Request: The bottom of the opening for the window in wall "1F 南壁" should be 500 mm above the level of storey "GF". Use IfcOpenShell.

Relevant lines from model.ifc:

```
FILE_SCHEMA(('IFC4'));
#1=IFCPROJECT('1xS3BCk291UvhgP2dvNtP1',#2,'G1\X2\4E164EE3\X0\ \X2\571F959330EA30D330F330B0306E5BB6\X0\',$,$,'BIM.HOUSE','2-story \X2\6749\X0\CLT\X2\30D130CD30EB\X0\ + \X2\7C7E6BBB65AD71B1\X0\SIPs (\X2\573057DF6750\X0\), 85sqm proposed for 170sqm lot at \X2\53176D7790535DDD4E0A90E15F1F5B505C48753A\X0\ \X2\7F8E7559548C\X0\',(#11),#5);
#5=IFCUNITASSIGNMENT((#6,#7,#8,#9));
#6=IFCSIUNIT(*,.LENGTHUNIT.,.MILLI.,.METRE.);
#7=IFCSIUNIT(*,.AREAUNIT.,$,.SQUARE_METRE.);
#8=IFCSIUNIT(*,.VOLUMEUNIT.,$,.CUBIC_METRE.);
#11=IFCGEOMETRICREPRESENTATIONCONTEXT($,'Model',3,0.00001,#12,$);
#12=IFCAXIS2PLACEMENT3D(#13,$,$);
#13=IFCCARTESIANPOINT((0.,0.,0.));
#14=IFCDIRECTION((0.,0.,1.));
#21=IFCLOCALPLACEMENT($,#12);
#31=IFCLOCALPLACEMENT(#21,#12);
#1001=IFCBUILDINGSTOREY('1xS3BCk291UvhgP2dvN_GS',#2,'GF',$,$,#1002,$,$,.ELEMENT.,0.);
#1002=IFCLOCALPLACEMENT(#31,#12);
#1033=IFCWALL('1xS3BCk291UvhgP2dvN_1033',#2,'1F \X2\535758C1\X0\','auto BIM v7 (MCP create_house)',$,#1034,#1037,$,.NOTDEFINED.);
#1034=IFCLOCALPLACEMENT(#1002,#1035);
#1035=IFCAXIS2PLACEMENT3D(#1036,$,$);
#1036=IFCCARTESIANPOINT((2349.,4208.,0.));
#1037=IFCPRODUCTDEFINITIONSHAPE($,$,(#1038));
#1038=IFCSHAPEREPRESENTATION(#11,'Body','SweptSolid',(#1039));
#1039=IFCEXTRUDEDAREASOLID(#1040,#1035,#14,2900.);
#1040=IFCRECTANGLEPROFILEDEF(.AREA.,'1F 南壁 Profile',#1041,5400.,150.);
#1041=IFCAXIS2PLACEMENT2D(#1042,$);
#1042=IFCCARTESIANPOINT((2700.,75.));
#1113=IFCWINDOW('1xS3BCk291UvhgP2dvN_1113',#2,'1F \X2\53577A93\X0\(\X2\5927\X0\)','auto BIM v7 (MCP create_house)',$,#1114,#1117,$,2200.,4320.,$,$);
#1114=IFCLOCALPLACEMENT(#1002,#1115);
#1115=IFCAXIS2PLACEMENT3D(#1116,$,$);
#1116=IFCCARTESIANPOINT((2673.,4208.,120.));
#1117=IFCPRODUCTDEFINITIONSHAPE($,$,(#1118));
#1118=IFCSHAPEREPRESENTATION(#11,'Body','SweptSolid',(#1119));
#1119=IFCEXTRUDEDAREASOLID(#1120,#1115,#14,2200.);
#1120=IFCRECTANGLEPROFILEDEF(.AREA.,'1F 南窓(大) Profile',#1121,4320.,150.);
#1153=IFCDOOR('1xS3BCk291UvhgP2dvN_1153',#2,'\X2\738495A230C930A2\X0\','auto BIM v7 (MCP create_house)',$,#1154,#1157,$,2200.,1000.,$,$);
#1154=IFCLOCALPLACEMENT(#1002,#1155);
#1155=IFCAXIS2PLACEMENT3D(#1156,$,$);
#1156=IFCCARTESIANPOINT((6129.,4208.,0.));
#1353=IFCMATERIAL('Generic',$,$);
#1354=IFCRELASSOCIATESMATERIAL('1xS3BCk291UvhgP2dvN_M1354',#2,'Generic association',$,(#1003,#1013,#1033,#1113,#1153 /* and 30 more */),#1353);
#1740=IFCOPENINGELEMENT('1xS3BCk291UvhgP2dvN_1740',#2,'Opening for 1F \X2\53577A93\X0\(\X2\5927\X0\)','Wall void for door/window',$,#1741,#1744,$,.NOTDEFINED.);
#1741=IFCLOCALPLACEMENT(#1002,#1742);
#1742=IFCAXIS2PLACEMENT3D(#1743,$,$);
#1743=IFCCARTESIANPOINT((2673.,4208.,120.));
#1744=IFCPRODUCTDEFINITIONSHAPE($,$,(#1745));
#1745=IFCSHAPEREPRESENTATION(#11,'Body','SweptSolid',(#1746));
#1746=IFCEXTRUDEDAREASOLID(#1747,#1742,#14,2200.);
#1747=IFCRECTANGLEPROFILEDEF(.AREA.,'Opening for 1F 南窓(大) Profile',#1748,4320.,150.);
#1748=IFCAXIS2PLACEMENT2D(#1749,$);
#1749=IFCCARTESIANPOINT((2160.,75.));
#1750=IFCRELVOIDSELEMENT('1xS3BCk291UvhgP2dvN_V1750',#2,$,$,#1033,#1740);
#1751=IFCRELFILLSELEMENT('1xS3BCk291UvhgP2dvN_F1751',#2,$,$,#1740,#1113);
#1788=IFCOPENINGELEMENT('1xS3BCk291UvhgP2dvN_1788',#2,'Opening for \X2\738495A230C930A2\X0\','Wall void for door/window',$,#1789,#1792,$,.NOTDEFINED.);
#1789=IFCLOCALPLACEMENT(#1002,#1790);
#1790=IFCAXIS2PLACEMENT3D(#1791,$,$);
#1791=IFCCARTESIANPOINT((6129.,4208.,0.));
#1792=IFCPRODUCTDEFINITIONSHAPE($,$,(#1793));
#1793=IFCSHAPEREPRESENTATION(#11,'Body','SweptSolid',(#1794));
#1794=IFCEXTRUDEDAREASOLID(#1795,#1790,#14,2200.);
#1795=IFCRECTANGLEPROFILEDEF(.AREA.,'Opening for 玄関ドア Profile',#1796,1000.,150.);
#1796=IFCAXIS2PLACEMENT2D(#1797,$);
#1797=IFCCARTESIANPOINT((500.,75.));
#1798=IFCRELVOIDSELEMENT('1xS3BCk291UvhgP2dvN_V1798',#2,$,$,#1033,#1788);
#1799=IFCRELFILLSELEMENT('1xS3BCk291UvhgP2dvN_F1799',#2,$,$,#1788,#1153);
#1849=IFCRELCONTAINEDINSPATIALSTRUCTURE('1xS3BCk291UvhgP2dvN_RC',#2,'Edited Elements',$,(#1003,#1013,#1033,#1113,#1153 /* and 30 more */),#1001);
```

```python
import numpy as np
import ifcopenshell
import ifcopenshell.api.geometry
import ifcopenshell.geom
import ifcopenshell.util.element
import ifcopenshell.util.placement
import ifcopenshell.util.shape
import ifcopenshell.util.unit

model = ifcopenshell.open("model.ifc")
unit_scale = ifcopenshell.util.unit.calculate_unit_scale(model)

window = model.by_id(1113)
opening = window.FillsVoids[0].RelatingOpeningElement
storey = ifcopenshell.util.element.get_container(window, ifc_class="IfcBuildingStorey")
level = ifcopenshell.util.placement.get_local_placement(storey.ObjectPlacement)[2, 3]

# The opening's origin need not be at the sill, so measure its lowest point.
shape = ifcopenshell.geom.create_shape(ifcopenshell.geom.settings(), opening)
bottom = ifcopenshell.util.shape.get_shape_bottom_elevation(shape, shape.geometry) / unit_scale
dz = level + 0.5 / unit_scale - bottom

shift = np.array([0.0, 0.0, dz])
# The window is not placed relative to its opening, so move both.
for product in (opening, window):
    matrix = ifcopenshell.util.placement.get_local_placement(product.ObjectPlacement)
    matrix[:3, 3] += shift
    ifcopenshell.api.geometry.edit_object_placement(model, product=product, matrix=matrix, is_si=False)

print(f"moved by {dz * unit_scale:+.3f} m")

model.write("model_rev.ifc")
```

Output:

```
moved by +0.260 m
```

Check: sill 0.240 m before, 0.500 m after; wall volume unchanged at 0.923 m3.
